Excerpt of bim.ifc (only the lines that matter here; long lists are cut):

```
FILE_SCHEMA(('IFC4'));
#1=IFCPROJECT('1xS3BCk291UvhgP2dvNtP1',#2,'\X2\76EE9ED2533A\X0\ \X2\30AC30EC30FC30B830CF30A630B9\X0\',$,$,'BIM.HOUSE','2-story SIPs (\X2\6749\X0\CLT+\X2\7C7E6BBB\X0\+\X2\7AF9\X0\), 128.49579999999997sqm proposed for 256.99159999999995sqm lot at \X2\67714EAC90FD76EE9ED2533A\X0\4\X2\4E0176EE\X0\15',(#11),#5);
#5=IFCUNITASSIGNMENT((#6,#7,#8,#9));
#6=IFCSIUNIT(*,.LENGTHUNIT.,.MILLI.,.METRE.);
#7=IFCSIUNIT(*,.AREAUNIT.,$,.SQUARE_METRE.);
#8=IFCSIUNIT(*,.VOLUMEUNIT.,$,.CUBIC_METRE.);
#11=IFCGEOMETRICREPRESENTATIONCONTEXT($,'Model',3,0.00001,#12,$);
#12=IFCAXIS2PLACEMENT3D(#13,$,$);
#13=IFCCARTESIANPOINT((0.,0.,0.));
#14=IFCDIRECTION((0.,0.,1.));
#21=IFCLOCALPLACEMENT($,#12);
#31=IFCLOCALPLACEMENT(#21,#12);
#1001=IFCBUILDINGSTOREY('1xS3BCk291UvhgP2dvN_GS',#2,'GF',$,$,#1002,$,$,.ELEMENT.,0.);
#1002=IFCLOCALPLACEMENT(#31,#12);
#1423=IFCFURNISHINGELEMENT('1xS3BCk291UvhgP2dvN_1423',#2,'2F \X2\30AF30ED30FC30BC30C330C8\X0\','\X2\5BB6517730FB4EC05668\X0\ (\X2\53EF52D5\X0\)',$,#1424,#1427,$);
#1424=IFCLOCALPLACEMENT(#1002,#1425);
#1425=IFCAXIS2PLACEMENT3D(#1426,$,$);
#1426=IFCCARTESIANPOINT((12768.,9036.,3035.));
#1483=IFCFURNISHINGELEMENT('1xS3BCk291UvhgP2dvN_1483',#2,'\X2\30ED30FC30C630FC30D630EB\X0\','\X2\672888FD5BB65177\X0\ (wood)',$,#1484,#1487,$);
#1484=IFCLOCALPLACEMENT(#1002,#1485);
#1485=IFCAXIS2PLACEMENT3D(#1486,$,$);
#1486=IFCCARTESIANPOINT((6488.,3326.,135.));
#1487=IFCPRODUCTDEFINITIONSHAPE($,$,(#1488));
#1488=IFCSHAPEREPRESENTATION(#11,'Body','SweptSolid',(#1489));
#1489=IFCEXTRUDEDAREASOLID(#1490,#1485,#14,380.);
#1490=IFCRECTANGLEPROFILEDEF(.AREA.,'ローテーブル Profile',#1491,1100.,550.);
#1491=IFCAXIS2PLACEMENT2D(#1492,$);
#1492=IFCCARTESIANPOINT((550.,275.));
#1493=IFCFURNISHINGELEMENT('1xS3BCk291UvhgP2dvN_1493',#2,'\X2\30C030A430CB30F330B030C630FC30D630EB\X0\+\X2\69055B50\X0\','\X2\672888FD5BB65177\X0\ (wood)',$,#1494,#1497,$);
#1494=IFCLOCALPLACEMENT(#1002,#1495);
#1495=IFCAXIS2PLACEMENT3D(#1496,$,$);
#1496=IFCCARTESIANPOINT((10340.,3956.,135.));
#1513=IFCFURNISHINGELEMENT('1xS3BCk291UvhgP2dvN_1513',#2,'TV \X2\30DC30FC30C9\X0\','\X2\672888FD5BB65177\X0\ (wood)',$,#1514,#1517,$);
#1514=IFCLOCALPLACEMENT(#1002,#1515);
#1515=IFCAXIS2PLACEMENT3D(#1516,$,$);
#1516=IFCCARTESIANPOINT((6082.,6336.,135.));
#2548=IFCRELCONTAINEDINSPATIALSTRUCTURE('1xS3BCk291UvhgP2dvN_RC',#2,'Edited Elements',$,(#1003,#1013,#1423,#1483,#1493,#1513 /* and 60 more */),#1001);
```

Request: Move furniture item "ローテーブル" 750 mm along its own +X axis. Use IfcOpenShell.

```python
import ifcopenshell
import ifcopenshell.api.geometry
import ifcopenshell.util.placement
import ifcopenshell.util.unit

model = ifcopenshell.open("bim.ifc")
unit_scale = ifcopenshell.util.unit.calculate_unit_scale(model)

item = model.by_guid("1xS3BCk291UvhgP2dvN_1483")
matrix = ifcopenshell.util.placement.get_local_placement(item.ObjectPlacement)
matrix[:3, 3] += matrix[:3, 0] * 0.75 / unit_scale
ifcopenshell.api.geometry.edit_object_placement(model, product=item, matrix=matrix, is_si=False)

print(ifcopenshell.util.placement.get_local_placement(item.ObjectPlacement).round(3) + 0.0)

model.write("bim_edited.ifc")
```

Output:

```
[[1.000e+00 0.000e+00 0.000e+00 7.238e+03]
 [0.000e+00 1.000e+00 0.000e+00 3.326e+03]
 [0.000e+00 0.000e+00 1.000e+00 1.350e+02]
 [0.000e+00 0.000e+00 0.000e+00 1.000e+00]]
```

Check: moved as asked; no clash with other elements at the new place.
